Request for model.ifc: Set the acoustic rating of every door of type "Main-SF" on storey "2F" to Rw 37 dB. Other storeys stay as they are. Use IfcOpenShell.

First a look at what the model holds.

```python
import ifcopenshell
import ifcopenshell.util.element

model = ifcopenshell.open("model.ifc")
print(model.schema)
storey = next(s for s in model.by_type("IfcBuildingStorey") if s.Name == "2F")
doors = [e for e in ifcopenshell.util.element.get_decomposition(storey) if e.is_a("IfcDoor")]
seen = {}
for e in doors:
    element_type = ifcopenshell.util.element.get_type(e)
    key = (element_type.Name if element_type != e and element_type else None, ifcopenshell.util.element.get_pset(e, "Pset_DoorCommon", "AcousticRating"))
    seen[key] = seen.get(key, 0) + 1
for (name, value), count in sorted(seen.items(), key=str):
    print(count, "x", name, "|", value)
```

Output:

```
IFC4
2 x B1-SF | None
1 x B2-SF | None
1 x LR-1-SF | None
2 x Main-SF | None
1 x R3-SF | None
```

```python
import ifcopenshell
import ifcopenshell.api.pset
import ifcopenshell.util.element

model = ifcopenshell.open("model.ifc")

storey = next(s for s in model.by_type("IfcBuildingStorey") if s.Name == "2F")
doors = [e for e in ifcopenshell.util.element.get_decomposition(storey) if e.is_a("IfcDoor")]

count = 0
for e in doors:
    element_type = ifcopenshell.util.element.get_type(e)
    if element_type in (None, e) or element_type.Name != "Main-SF":
        continue
    # add_pset returns the element's existing set when there is one.
    pset = ifcopenshell.api.pset.add_pset(model, product=e, name="Pset_DoorCommon")
    ifcopenshell.api.pset.edit_pset(model, pset=pset, properties={"AcousticRating": "Rw 37 dB"})
    count += 1

print(count, "doors updated")

model.write("model_updated.ifc")
```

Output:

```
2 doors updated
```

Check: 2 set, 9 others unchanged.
